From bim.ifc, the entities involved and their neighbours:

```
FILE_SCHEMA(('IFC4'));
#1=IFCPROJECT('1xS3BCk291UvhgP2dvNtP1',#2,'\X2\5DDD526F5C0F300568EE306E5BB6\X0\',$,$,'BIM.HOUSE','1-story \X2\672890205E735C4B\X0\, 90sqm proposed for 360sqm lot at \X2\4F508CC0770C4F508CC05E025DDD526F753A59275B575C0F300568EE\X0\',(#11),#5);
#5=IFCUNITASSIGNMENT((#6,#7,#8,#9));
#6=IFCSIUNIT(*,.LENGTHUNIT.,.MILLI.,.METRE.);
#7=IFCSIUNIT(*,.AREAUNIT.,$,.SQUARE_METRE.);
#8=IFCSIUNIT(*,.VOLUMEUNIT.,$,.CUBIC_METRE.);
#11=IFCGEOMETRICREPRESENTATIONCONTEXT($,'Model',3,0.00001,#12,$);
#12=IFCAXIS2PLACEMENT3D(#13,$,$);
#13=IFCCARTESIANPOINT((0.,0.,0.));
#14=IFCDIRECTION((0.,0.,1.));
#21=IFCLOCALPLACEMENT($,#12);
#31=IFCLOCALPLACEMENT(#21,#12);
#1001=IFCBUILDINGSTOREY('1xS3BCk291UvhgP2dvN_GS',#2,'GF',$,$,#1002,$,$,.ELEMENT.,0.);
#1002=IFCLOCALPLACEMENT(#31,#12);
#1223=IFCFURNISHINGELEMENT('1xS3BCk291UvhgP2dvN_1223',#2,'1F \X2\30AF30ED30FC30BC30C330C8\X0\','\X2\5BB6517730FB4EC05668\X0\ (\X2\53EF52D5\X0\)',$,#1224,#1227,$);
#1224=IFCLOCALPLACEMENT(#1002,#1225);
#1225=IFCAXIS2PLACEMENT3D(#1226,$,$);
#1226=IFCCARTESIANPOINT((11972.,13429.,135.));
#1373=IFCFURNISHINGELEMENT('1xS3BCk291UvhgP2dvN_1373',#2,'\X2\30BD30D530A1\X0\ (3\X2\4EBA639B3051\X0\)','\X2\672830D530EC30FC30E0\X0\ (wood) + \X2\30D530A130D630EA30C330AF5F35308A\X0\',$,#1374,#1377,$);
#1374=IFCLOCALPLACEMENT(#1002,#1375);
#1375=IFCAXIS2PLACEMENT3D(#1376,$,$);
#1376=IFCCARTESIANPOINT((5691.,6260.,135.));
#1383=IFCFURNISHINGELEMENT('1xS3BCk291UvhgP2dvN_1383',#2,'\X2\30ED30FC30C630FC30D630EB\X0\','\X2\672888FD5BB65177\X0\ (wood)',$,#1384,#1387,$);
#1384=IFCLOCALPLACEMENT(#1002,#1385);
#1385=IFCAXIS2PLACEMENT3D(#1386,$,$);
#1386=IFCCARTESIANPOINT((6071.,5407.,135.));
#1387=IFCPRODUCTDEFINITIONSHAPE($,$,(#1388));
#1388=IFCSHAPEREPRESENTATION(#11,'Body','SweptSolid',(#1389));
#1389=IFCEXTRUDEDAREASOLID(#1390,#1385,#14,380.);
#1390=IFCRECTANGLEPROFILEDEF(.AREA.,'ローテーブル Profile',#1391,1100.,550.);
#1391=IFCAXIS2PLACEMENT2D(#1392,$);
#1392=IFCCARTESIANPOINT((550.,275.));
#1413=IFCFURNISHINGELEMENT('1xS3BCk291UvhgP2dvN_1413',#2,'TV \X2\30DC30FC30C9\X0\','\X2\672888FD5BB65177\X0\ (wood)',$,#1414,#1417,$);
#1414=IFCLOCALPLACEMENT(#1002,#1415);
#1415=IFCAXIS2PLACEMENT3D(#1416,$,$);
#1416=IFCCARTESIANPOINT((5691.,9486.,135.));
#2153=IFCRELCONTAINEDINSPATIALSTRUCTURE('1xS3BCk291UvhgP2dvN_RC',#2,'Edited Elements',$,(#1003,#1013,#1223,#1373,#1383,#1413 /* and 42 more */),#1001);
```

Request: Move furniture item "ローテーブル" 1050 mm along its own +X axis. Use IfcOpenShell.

```python
import ifcopenshell
import ifcopenshell.api.geometry
import ifcopenshell.util.placement
import ifcopenshell.util.unit

model = ifcopenshell.open("bim.ifc")
unit_scale = ifcopenshell.util.unit.calculate_unit_scale(model)

item = model.by_guid("1xS3BCk291UvhgP2dvN_1383")
matrix = ifcopenshell.util.placement.get_local_placement(item.ObjectPlacement)
matrix[:3, 3] += matrix[:3, 0] * 1.05 / unit_scale
ifcopenshell.api.geometry.edit_object_placement(model, product=item, matrix=matrix, is_si=False)

print(ifcopenshell.util.placement.get_local_placement(item.ObjectPlacement).round(3) + 0.0)

model.write("bim_updated.ifc")
```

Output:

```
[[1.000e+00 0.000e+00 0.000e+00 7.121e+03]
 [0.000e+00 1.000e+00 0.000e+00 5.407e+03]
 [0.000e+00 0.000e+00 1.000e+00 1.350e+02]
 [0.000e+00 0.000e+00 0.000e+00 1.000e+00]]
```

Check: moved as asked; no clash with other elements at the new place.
